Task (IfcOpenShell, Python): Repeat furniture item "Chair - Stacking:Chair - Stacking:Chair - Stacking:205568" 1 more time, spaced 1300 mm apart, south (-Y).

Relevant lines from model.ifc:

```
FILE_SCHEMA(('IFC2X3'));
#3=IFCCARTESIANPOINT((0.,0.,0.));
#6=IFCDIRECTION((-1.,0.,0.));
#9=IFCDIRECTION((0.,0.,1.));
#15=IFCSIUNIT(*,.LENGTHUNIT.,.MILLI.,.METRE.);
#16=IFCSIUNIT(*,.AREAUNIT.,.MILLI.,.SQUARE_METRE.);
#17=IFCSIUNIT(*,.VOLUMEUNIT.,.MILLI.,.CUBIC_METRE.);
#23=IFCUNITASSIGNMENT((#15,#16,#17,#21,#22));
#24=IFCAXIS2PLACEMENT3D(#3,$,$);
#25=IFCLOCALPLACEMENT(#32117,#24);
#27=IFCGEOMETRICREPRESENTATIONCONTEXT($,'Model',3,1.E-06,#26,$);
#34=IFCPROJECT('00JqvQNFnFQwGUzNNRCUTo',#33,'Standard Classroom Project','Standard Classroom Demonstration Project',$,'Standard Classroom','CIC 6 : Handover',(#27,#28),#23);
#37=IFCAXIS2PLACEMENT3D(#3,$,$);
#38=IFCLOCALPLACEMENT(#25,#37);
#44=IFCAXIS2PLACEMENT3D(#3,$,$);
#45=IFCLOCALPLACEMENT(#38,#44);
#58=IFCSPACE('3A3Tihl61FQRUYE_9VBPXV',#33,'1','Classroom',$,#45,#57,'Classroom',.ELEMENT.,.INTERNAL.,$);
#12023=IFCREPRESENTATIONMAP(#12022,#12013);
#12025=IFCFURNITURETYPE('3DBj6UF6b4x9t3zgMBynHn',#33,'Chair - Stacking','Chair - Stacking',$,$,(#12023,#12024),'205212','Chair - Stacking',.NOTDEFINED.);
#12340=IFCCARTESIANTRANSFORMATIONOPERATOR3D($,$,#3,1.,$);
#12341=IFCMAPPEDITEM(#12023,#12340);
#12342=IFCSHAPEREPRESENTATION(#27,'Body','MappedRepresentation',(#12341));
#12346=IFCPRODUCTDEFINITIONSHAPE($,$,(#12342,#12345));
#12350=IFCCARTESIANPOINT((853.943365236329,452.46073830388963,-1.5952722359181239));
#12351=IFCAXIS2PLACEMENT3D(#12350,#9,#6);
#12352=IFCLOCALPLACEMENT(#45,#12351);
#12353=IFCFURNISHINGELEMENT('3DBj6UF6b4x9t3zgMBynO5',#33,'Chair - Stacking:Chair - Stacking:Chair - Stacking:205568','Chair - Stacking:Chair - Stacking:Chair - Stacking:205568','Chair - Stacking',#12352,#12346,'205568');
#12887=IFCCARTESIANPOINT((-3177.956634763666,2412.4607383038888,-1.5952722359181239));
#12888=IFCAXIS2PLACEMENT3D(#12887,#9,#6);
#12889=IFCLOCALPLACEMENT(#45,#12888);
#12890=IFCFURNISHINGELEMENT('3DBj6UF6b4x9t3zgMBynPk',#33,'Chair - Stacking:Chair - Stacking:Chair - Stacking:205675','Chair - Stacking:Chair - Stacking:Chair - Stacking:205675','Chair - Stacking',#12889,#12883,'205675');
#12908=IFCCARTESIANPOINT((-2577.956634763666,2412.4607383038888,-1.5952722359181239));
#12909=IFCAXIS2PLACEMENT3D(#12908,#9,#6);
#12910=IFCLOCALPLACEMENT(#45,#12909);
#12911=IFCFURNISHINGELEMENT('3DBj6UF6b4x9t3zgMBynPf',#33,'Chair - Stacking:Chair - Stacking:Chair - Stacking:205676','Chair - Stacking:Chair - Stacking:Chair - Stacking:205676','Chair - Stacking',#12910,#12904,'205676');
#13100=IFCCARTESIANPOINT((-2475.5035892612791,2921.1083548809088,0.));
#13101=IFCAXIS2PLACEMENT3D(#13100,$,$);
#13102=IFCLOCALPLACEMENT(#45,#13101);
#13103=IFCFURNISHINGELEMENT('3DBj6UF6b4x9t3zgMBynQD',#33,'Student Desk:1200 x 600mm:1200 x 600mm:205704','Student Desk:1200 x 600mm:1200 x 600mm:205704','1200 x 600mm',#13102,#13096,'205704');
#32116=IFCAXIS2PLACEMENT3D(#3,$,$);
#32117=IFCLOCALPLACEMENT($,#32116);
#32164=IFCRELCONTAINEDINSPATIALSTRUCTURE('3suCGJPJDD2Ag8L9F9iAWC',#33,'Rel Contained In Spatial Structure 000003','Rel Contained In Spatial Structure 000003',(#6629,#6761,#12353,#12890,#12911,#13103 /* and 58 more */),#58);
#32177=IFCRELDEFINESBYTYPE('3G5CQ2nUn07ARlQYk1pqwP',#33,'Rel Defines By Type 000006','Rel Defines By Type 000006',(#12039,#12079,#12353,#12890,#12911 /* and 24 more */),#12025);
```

```python
import numpy as np
import ifcopenshell
import ifcopenshell.api.geometry
import ifcopenshell.api.root
import ifcopenshell.util.element
import ifcopenshell.util.placement

model = ifcopenshell.open("model.ifc")


def reuse_history(source, copy):
    """copy_class also copies each property set's owner history, people and application; keep the originals."""
    for rel in copy.IsDefinedBy:
        if rel.is_a("IfcRelDefinesByProperties") and (history := rel.RelatingPropertyDefinition.OwnerHistory):
            rel.RelatingPropertyDefinition.OwnerHistory = source.OwnerHistory
            ifcopenshell.util.element.remove_deep2(model, history)


source = model.by_guid("3DBj6UF6b4x9t3zgMBynO5")
base = ifcopenshell.util.placement.get_local_placement(source.ObjectPlacement)
step = np.array([0.0, -1.0, 0.0]) * 1300.0

for i in range(1, 2):
    copy = ifcopenshell.api.root.copy_class(model, product=source)
    copy.Representation = ifcopenshell.util.element.copy_deep(
        model, source.Representation, exclude=["IfcGeometricRepresentationContext", "IfcRepresentationMap"]
    )
    copy.Name = "Chair - Stacking:Chair - Stacking:Chair - Stacking"
    copy.Tag = None
    reuse_history(source, copy)
    matrix = base.copy()
    matrix[:3, 3] += i * step
    print("added at", matrix[:3, 3].round(3) + 0.0)
    ifcopenshell.api.geometry.edit_object_placement(model, product=copy, matrix=matrix, is_si=False)

model.write("model_edited.ifc")
```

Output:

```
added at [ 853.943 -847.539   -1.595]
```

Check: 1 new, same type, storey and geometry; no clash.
